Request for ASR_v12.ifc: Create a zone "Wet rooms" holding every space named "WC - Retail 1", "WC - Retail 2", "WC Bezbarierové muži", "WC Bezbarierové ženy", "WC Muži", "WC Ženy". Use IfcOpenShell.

First a look at what the model holds.

```python
import ifcopenshell

model = ifcopenshell.open("ASR_v12.ifc")
print(model.schema)
seen = {}
for space in model.by_type("IfcSpace"):
    seen[space.LongName] = seen.get(space.LongName, 0) + 1
for name, count in sorted(seen.items(), key=str):
    print(count, "x", name)
print("zones:", [z.Name for z in model.by_type("IfcZone")][:20])
```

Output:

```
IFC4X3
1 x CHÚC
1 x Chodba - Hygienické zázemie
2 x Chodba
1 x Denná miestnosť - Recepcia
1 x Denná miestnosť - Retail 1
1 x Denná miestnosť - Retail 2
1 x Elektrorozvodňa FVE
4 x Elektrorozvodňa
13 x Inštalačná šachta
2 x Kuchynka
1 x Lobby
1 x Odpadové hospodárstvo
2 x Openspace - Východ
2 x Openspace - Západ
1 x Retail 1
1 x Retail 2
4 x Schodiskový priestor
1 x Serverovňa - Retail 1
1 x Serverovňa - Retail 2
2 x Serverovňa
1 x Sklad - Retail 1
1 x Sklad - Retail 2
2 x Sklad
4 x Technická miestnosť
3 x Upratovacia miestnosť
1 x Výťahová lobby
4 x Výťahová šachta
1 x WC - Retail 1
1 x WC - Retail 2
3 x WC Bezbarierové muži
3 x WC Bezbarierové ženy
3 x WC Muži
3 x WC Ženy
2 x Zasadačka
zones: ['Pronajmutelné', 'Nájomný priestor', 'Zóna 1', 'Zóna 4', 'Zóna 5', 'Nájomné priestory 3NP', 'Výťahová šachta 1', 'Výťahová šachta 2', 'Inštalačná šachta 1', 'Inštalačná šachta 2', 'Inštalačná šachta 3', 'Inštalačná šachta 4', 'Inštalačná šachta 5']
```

```python
import ifcopenshell
import ifcopenshell.api.group
import ifcopenshell.api.root

model = ifcopenshell.open("ASR_v12.ifc")

names = {"WC - Retail 1", "WC - Retail 2", "WC Bezbarierové muži", "WC Bezbarierové ženy", "WC Muži", "WC Ženy"}
spaces = [s for s in model.by_type("IfcSpace") if s.LongName in names]

zone = ifcopenshell.api.root.create_entity(model, ifc_class="IfcZone", name="Wet rooms")
ifcopenshell.api.group.assign_group(model, products=spaces, group=zone)
print(len(spaces), "spaces in", zone.Name)

model.write("ASR_v12_v2.ifc")
```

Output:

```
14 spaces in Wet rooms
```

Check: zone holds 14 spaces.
